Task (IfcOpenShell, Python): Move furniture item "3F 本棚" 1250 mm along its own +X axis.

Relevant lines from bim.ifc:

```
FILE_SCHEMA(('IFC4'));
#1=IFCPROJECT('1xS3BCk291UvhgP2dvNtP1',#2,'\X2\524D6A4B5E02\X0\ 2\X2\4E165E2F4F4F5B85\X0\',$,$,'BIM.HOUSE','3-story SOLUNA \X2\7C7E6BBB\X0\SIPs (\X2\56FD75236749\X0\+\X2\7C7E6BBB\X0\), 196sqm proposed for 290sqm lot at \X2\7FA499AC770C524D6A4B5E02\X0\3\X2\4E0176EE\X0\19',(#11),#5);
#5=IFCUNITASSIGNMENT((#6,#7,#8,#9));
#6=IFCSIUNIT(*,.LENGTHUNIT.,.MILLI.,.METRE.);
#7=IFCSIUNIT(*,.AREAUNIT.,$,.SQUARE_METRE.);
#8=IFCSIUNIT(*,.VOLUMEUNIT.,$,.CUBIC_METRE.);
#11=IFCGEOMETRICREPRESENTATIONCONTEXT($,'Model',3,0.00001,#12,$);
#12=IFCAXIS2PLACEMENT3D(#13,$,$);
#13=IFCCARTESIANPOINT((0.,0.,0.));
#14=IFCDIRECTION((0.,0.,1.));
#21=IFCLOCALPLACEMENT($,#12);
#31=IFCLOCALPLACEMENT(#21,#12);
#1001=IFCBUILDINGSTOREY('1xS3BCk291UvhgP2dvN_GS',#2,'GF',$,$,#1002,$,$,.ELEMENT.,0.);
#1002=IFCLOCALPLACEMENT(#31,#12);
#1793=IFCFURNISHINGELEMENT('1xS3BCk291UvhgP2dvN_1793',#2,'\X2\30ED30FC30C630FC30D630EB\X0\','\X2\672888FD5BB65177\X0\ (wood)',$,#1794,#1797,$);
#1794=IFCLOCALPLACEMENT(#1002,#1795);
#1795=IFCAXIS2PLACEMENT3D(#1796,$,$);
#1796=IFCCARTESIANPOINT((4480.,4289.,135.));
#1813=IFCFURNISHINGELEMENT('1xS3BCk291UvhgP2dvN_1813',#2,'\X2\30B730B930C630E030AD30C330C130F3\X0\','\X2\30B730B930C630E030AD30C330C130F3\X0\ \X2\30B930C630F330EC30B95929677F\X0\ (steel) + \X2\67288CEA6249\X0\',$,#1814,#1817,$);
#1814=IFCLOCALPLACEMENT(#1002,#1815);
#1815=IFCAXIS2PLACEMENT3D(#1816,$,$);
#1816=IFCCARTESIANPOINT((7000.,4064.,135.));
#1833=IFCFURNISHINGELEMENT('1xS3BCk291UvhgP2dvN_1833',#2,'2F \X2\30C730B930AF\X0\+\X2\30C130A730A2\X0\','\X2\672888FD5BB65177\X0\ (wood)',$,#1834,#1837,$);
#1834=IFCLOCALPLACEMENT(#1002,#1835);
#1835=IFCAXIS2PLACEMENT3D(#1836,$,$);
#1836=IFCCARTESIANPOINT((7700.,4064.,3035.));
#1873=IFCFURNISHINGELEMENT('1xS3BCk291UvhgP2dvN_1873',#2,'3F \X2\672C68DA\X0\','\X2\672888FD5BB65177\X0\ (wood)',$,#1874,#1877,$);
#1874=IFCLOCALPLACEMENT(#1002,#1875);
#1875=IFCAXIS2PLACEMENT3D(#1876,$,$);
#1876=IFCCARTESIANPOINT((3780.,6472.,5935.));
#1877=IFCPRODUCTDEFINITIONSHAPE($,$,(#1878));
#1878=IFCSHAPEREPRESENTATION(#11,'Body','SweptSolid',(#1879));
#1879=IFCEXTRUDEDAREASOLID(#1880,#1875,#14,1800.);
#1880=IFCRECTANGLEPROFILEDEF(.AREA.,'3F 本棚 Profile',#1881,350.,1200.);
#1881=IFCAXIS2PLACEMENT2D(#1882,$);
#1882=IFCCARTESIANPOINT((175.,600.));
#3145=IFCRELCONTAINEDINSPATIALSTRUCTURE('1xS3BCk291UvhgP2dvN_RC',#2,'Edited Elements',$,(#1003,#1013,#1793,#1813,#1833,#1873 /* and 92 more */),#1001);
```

```python
import ifcopenshell
import ifcopenshell.api.geometry
import ifcopenshell.util.placement
import ifcopenshell.util.unit

model = ifcopenshell.open("bim.ifc")
unit_scale = ifcopenshell.util.unit.calculate_unit_scale(model)

item = model.by_guid("1xS3BCk291UvhgP2dvN_1873")
matrix = ifcopenshell.util.placement.get_local_placement(item.ObjectPlacement)
matrix[:3, 3] += matrix[:3, 0] * 1.25 / unit_scale
ifcopenshell.api.geometry.edit_object_placement(model, product=item, matrix=matrix, is_si=False)

print(ifcopenshell.util.placement.get_local_placement(item.ObjectPlacement).round(3) + 0.0)

model.write("bim_updated.ifc")
```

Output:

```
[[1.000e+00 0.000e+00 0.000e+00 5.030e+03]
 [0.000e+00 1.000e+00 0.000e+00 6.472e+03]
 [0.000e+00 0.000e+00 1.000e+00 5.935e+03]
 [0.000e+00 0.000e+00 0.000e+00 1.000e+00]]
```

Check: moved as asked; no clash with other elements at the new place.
